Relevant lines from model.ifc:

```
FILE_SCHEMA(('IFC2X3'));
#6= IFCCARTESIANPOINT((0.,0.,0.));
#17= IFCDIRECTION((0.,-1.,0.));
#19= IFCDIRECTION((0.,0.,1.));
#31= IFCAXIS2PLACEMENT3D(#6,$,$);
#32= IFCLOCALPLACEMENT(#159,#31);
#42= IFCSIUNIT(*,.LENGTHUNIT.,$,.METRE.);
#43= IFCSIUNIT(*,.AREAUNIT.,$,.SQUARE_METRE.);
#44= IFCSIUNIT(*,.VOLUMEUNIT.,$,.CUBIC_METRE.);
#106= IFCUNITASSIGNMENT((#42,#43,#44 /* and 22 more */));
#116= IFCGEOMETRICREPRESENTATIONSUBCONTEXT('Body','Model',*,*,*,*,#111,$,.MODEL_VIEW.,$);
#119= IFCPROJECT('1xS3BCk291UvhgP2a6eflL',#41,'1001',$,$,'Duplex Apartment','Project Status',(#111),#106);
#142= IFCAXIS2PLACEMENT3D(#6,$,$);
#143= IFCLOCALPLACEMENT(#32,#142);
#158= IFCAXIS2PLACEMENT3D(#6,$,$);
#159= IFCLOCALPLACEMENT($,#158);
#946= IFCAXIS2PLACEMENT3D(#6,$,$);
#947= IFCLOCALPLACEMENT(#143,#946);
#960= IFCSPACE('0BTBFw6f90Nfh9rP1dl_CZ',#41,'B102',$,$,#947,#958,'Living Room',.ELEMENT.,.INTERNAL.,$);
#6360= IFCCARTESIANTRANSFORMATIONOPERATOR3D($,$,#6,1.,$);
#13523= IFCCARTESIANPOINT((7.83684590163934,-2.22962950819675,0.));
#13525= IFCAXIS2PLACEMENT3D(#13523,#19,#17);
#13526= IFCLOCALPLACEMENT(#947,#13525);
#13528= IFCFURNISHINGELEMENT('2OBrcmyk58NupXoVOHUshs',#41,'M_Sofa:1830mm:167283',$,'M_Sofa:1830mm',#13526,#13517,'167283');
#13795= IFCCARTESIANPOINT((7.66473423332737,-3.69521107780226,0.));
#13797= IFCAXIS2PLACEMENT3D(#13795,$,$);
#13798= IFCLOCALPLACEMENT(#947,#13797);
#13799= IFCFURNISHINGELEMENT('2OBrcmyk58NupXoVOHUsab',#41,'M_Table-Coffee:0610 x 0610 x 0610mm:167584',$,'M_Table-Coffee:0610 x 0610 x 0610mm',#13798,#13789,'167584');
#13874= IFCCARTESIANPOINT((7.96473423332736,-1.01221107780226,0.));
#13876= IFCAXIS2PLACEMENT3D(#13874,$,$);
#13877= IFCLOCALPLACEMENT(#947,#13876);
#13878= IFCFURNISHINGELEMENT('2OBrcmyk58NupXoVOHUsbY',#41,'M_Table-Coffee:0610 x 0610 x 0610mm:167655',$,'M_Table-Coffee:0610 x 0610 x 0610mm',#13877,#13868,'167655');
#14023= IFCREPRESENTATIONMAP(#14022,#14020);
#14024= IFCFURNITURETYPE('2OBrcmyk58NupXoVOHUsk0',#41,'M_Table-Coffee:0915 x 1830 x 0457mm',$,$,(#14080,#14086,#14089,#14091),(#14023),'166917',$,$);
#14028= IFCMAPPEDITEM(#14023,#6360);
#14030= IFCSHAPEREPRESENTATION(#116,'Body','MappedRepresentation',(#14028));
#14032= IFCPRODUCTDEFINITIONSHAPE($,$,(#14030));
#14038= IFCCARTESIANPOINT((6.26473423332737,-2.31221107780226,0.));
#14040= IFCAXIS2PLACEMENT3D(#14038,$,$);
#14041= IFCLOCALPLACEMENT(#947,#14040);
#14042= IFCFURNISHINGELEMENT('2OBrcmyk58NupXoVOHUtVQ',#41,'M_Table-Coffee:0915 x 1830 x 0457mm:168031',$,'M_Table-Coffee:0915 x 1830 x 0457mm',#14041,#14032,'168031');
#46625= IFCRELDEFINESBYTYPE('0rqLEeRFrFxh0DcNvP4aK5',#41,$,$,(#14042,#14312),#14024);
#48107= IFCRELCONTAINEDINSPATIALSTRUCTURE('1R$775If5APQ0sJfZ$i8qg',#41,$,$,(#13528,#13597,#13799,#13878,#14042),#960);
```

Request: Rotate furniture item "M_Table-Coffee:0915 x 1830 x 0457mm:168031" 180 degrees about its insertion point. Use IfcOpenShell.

```python
import ifcopenshell
import ifcopenshell.api.geometry
import ifcopenshell.util.placement

model = ifcopenshell.open("model.ifc")

item = model.by_guid("2OBrcmyk58NupXoVOHUtVQ")
matrix = ifcopenshell.util.placement.get_local_placement(item.ObjectPlacement)
matrix = matrix @ ifcopenshell.util.placement.rotation(180, "Z")
ifcopenshell.api.geometry.edit_object_placement(model, product=item, matrix=matrix, is_si=False)

print(ifcopenshell.util.placement.get_local_placement(item.ObjectPlacement).round(3) + 0.0)

model.write("model-out.ifc")
```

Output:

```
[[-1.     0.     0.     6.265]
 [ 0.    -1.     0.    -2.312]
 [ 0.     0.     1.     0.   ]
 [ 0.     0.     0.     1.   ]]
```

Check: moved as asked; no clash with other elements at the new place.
